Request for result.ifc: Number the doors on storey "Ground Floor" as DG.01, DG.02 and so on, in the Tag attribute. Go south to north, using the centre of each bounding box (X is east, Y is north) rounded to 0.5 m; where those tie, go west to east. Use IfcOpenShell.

First a look at what the model holds.

```python
import ifcopenshell
import ifcopenshell.util.element
import ifcopenshell.util.placement

model = ifcopenshell.open("result.ifc")
print(model.schema)
storey = next(s for s in model.by_type("IfcBuildingStorey") if s.Name == "Ground Floor")
doors = [e for e in ifcopenshell.util.element.get_decomposition(storey) if e.is_a("IfcDoor")]
for e in sorted(doors, key=lambda e: e.id()):
    origin = ifcopenshell.util.placement.get_local_placement(e.ObjectPlacement)[:3, 3]
    print(e.id(), e.Tag, e.Name, origin.round(2) + 0.0, sep=" | ")
```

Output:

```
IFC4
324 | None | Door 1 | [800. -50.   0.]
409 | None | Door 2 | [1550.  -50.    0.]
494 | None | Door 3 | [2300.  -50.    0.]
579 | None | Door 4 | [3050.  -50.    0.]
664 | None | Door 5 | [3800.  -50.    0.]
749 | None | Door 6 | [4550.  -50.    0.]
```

```python
import ifcopenshell
import ifcopenshell.geom
import ifcopenshell.util.element
import ifcopenshell.util.shape

model = ifcopenshell.open("result.ifc")
settings = ifcopenshell.geom.settings()
settings.set("use-world-coords", True)


def centre(element):
    shape = ifcopenshell.geom.create_shape(settings, element)
    return ifcopenshell.util.shape.get_bbox_centroid(shape.geometry)


storey = next(s for s in model.by_type("IfcBuildingStorey") if s.Name == "Ground Floor")
doors = [e for e in ifcopenshell.util.element.get_decomposition(storey) if e.is_a("IfcDoor")]

# Insertion points can sit at a corner or the storey origin, so sort by the geometry (in metres).
centres = {e: centre(e) for e in doors}
doors.sort(key=lambda e: (round(centres[e][1] / 0.5), centres[e][0]))

for i, e in enumerate(doors, start=1):
    number = f"DG.{i:02d}"
    e.Tag = number
    print(e.id(), number)

model.write("result_updated.ifc")
```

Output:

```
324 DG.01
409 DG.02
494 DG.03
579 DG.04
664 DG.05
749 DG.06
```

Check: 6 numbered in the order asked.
